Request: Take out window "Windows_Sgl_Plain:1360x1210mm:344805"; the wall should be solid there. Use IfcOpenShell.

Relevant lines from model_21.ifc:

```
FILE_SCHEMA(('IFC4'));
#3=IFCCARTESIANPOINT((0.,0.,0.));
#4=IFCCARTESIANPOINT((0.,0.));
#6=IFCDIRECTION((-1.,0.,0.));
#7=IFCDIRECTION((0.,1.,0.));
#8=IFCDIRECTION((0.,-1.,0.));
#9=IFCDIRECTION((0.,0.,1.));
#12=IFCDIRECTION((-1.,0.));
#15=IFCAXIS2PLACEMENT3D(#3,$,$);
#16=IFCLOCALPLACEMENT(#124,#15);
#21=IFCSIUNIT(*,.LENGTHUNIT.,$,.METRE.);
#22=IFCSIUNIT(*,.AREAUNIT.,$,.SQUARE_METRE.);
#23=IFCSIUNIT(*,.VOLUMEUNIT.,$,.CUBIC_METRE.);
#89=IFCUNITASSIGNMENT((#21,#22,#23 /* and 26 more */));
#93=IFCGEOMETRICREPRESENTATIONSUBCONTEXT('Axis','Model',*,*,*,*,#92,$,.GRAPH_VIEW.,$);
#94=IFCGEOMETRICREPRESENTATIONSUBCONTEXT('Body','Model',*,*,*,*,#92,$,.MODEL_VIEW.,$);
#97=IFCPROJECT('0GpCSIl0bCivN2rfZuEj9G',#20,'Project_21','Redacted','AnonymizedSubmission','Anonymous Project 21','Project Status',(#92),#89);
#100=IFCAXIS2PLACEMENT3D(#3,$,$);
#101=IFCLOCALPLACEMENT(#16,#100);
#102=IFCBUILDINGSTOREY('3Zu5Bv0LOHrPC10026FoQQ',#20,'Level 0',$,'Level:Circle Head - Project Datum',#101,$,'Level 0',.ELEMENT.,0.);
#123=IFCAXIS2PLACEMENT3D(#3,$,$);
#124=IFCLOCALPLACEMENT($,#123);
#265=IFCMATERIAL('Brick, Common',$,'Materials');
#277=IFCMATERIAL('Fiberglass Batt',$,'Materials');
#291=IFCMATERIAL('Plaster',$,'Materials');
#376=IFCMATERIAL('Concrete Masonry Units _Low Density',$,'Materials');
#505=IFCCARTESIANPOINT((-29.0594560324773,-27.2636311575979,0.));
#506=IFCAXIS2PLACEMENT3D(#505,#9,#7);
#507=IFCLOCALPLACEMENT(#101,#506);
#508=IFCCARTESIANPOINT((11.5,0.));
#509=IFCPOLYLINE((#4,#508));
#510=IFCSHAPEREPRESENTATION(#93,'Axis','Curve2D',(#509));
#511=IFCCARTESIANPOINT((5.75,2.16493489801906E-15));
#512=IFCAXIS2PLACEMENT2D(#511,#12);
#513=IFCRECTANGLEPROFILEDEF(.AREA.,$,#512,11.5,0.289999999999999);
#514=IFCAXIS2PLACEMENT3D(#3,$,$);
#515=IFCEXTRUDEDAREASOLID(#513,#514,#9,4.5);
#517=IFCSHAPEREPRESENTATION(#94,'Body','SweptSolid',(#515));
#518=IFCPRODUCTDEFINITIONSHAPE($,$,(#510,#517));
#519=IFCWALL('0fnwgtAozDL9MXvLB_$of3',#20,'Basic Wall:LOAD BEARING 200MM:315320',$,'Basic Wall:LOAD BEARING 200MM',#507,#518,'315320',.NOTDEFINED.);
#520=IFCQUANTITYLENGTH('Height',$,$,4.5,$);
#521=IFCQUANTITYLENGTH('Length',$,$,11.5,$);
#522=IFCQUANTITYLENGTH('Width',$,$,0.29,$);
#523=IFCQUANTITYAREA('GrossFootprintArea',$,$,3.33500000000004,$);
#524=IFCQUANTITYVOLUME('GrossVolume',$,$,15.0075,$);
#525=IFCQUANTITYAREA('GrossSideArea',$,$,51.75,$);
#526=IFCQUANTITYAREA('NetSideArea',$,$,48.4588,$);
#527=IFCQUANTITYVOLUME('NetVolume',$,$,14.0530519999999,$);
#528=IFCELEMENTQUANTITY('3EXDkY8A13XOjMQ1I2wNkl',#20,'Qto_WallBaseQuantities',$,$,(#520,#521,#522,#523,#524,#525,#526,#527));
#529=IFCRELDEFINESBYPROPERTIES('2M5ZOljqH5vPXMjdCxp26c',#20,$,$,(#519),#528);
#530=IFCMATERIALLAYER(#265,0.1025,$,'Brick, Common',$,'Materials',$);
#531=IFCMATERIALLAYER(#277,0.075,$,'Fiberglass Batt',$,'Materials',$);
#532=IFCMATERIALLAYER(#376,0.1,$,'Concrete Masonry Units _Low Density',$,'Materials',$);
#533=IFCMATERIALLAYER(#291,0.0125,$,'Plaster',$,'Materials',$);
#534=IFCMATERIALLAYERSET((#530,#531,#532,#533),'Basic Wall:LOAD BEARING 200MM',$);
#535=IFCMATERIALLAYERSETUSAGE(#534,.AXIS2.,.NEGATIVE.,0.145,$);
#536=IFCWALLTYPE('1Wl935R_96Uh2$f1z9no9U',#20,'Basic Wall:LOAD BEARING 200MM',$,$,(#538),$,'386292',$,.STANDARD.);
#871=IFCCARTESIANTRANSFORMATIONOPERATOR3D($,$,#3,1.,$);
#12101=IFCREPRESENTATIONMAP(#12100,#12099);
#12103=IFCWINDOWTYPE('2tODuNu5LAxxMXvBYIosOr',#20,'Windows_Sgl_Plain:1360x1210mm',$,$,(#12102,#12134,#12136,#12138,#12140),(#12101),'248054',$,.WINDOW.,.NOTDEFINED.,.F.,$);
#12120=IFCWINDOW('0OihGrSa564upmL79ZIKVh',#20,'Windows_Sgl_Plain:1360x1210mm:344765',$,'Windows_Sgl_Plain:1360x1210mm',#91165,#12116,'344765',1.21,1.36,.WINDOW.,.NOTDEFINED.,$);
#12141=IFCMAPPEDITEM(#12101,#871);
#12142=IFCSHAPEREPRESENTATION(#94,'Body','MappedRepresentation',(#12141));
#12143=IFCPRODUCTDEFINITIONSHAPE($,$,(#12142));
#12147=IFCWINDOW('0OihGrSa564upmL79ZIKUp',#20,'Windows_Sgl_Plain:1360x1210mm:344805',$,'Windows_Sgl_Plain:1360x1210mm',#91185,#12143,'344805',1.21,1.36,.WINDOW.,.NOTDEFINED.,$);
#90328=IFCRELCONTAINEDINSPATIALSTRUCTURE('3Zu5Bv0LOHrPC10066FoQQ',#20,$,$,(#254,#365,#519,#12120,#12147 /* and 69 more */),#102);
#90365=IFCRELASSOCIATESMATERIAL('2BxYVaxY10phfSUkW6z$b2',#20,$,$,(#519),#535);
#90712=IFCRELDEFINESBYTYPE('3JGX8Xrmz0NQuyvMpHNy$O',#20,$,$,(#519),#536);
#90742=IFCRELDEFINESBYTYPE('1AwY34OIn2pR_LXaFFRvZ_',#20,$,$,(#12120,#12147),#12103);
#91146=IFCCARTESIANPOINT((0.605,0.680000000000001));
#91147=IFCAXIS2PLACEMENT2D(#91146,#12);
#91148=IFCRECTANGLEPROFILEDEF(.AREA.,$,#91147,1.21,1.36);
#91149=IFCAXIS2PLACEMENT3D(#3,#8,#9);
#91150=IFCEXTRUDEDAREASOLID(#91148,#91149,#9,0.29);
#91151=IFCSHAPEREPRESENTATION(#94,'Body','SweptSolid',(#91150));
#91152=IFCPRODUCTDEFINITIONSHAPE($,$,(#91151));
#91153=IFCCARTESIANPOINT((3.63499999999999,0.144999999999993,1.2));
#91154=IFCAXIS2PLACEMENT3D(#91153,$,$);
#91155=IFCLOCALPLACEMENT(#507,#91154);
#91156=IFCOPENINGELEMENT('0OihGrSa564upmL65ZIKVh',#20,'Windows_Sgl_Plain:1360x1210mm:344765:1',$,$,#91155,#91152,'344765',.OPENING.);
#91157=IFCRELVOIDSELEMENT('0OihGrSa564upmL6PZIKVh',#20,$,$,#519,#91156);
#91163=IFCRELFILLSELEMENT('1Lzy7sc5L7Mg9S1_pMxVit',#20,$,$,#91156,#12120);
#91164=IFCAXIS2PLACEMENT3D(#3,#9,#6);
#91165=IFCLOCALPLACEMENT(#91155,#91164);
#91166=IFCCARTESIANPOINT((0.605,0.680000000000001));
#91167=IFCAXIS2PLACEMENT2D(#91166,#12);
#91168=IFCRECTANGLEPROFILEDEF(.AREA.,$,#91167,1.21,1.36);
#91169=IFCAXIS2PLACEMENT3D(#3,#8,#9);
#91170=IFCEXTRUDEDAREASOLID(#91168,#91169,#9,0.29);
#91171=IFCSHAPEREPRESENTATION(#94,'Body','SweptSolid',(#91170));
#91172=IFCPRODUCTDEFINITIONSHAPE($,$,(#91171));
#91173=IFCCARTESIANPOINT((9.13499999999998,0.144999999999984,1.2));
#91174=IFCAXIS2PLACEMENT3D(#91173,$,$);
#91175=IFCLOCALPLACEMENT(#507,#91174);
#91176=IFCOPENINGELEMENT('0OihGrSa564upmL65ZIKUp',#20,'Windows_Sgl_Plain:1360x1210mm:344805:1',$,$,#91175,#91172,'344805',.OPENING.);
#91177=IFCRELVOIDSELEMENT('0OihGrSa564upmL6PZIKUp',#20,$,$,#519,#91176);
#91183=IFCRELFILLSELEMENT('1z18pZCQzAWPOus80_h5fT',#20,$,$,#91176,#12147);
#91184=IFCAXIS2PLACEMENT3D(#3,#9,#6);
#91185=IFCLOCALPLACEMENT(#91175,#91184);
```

```python
import ifcopenshell
import ifcopenshell.api.feature
import ifcopenshell.api.pset
import ifcopenshell.api.root
import ifcopenshell.geom
import ifcopenshell.util.element
import ifcopenshell.util.shape
import ifcopenshell.util.unit

model = ifcopenshell.open("model_21.ifc")
area_scale = ifcopenshell.util.unit.calculate_unit_scale(model, "AREAUNIT")
volume_scale = ifcopenshell.util.unit.calculate_unit_scale(model, "VOLUMEUNIT")
settings = ifcopenshell.geom.settings()


def volume(element):
    """Net volume in cubic metres, openings subtracted."""
    shape = ifcopenshell.geom.create_shape(settings, element)
    return ifcopenshell.util.shape.get_volume(shape.geometry)


window = model.by_id(12147)
opening = window.FillsVoids[0].RelatingOpeningElement
wall = opening.VoidsElements[0].RelatingBuildingElement
before = volume(wall)

ifcopenshell.api.root.remove_product(model, product=window)
ifcopenshell.api.feature.remove_feature(model, feature=opening)

after = volume(wall)
thickness = 0.29  # wall thickness in metres

# Update the wall's stored quantities.
qto = model.by_id(ifcopenshell.util.element.get_pset(wall, "Qto_WallBaseQuantities", should_inherit=False)["id"])
ifcopenshell.api.pset.edit_qto(model, qto=qto, properties={
    "NetSideArea": after / thickness / area_scale,
    "NetVolume": after / volume_scale,
})

print(f"wall volume {before:.3f} -> {after:.3f} m3")

model.write("model_21_rev.ifc")
```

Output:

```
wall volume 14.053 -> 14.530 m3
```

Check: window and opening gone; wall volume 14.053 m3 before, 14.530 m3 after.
